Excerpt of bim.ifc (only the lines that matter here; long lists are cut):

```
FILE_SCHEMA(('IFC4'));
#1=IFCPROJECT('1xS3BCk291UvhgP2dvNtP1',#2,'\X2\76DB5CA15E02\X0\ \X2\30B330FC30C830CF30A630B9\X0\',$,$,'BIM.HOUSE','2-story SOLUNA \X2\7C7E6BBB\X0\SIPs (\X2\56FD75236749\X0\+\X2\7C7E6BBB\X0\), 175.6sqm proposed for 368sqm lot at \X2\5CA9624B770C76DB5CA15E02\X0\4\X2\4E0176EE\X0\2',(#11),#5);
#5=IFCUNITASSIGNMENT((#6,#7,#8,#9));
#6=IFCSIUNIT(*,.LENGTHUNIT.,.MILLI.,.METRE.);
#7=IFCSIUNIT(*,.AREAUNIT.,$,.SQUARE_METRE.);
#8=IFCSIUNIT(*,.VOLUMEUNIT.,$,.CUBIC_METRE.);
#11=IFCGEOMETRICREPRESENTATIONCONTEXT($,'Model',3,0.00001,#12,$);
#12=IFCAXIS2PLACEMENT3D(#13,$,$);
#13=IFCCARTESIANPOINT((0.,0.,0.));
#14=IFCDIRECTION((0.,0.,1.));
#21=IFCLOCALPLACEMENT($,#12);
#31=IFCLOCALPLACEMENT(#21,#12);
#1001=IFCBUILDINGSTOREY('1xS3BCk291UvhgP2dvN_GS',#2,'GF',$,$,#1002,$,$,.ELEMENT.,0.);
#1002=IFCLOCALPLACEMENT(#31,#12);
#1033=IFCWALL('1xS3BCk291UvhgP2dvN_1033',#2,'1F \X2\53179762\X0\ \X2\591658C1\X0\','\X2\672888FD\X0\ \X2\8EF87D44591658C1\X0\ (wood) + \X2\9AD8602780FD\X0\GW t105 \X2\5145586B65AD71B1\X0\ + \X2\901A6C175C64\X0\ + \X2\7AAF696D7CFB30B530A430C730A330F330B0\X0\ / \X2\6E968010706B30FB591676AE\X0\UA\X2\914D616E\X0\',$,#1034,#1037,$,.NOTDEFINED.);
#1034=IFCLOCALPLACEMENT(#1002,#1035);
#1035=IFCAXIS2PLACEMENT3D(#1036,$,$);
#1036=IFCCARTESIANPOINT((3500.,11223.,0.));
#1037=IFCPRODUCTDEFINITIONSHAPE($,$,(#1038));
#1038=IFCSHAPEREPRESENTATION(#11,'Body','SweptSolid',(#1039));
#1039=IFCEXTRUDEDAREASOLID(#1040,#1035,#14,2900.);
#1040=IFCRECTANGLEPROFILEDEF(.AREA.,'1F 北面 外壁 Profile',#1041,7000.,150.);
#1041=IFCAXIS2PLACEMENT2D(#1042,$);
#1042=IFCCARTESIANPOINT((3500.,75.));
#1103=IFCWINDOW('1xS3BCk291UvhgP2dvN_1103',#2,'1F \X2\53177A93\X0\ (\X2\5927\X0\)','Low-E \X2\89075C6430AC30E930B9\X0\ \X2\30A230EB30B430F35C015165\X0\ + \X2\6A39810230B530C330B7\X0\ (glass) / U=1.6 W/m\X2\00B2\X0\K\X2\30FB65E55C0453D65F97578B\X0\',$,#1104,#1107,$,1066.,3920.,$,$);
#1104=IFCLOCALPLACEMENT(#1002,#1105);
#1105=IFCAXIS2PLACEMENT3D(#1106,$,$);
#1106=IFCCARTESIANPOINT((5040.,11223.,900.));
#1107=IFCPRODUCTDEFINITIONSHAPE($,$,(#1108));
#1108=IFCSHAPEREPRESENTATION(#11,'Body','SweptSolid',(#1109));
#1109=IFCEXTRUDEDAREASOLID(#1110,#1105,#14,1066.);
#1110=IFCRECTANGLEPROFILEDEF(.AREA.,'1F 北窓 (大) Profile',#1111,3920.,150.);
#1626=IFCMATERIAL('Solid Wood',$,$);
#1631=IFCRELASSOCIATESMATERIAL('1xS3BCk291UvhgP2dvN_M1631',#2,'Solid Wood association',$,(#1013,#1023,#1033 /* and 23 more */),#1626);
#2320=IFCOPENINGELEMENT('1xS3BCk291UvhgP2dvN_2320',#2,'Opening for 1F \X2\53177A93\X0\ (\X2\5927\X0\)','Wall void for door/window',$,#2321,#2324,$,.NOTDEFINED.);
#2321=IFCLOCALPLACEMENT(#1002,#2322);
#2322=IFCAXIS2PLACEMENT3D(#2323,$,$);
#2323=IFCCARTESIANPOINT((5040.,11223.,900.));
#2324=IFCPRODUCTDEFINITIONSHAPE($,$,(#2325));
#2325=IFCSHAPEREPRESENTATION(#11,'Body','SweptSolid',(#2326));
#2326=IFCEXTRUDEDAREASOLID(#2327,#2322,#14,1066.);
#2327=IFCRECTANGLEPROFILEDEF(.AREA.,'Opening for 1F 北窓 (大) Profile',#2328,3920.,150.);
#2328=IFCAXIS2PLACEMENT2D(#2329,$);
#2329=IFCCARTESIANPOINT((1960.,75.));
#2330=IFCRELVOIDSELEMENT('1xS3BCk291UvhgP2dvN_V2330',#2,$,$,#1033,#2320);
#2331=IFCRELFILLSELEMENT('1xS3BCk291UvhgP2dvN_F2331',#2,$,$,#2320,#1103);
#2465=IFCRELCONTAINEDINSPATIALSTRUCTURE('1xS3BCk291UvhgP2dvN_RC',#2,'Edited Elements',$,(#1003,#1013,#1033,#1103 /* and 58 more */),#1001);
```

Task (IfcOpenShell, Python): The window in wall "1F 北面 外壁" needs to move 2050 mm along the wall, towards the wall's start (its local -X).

```python
import ifcopenshell
import ifcopenshell.api.geometry
import ifcopenshell.util.placement

model = ifcopenshell.open("bim.ifc")

window = model.by_guid("1xS3BCk291UvhgP2dvN_1103")
opening = window.FillsVoids[0].RelatingOpeningElement
wall = opening.VoidsElements[0].RelatingBuildingElement

wall_matrix = ifcopenshell.util.placement.get_local_placement(wall.ObjectPlacement)
shift = wall_matrix[:3, 0] * -2050.0
before = ifcopenshell.util.placement.get_local_placement(window.ObjectPlacement)[:3, 3].copy()

# The window is not placed relative to its opening, so move both.
for product in (opening, window):
    matrix = ifcopenshell.util.placement.get_local_placement(product.ObjectPlacement)
    matrix[:3, 3] += shift
    ifcopenshell.api.geometry.edit_object_placement(model, product=product, matrix=matrix, is_si=False)

after = ifcopenshell.util.placement.get_local_placement(window.ObjectPlacement)[:3, 3]
print("window moved by", (after - before).round(3) + 0.0)

model.write("bim_edited.ifc")
```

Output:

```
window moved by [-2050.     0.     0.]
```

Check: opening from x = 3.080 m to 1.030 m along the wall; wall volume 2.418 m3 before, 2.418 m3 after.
